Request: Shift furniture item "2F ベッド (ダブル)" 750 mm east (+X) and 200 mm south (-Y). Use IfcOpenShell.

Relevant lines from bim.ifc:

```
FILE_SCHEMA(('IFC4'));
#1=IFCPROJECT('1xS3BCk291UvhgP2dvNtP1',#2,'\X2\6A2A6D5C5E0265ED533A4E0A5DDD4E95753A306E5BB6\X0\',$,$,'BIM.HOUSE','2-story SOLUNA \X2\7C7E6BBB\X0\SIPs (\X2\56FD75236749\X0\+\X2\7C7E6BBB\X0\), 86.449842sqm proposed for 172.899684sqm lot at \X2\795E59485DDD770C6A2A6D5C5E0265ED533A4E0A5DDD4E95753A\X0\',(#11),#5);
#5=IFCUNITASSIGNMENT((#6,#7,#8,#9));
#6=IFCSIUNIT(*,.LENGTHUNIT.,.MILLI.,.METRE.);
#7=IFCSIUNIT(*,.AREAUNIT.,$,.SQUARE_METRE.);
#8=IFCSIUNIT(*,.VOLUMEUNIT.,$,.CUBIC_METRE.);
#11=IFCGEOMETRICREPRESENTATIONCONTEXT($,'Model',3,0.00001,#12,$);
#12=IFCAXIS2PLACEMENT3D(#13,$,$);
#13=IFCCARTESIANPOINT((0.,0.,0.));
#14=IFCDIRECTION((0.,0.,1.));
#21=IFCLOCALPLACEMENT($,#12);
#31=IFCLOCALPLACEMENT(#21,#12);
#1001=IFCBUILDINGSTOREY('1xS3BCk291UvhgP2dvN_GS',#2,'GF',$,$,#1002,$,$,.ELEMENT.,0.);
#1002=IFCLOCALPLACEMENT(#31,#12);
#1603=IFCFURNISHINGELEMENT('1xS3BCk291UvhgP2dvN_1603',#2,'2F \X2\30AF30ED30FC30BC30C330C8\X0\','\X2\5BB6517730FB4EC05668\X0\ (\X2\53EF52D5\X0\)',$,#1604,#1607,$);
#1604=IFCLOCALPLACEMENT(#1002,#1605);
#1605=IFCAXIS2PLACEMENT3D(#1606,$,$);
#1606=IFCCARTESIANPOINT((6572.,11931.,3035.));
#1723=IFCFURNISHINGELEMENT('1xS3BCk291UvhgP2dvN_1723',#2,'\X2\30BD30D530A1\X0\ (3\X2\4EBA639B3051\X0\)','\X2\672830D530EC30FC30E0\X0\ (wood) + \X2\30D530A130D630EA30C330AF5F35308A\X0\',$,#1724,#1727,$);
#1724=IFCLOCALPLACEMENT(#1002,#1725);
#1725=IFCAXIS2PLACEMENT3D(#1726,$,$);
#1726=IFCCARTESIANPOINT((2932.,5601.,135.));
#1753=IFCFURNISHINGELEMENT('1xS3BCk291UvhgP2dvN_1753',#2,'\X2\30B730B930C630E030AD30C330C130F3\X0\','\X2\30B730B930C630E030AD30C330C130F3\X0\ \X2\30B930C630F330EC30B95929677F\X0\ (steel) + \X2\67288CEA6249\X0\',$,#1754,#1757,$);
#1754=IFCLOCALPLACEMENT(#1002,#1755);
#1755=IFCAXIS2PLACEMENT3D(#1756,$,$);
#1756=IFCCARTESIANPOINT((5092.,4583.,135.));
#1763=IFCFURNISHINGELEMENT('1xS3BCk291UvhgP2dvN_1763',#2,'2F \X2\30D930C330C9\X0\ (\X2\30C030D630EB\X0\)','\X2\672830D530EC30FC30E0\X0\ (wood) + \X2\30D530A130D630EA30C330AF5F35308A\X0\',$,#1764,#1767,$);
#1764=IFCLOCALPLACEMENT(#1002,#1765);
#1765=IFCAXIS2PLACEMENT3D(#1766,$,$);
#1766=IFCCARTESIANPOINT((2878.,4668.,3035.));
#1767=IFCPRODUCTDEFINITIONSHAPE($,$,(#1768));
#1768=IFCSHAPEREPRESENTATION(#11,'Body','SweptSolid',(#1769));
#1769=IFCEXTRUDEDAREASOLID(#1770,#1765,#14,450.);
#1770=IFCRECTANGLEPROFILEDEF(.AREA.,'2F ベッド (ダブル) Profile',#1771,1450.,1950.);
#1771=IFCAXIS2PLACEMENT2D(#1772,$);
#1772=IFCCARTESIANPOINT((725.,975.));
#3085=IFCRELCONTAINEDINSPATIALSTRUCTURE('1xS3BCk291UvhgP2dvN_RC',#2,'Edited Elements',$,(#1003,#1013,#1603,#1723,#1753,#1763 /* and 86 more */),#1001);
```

```python
import ifcopenshell
import ifcopenshell.api.geometry
import ifcopenshell.util.placement
import ifcopenshell.util.unit

model = ifcopenshell.open("bim.ifc")
unit_scale = ifcopenshell.util.unit.calculate_unit_scale(model)

item = model.by_guid("1xS3BCk291UvhgP2dvN_1763")
matrix = ifcopenshell.util.placement.get_local_placement(item.ObjectPlacement)
matrix[0, 3] += 0.75 / unit_scale
matrix[1, 3] -= 0.2 / unit_scale
ifcopenshell.api.geometry.edit_object_placement(model, product=item, matrix=matrix, is_si=False)

print(ifcopenshell.util.placement.get_local_placement(item.ObjectPlacement).round(3) + 0.0)

model.write("bim_updated.ifc")
```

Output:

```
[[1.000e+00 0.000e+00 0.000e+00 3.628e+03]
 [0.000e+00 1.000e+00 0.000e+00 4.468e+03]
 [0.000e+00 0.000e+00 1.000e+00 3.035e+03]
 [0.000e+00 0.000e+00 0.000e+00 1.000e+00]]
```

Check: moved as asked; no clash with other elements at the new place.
